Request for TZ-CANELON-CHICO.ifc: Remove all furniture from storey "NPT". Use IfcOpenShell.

First a look at what the model holds.

```python
import ifcopenshell
import ifcopenshell.util.element

model = ifcopenshell.open("TZ-CANELON-CHICO.ifc")
print(model.schema)
storey = next(s for s in model.by_type("IfcBuildingStorey") if s.Name == "NPT")
furniture = [e for e in ifcopenshell.util.element.get_decomposition(storey) if e.is_a("IfcFurnishingElement")]
seen = {}
for e in furniture:
    element_type = ifcopenshell.util.element.get_type(e)
    name = element_type.Name if element_type not in (None, e) else None
    seen[name] = seen.get(name, 0) + 1
for name, count in sorted(seen.items(), key=str):
    print(count, "x", name)
```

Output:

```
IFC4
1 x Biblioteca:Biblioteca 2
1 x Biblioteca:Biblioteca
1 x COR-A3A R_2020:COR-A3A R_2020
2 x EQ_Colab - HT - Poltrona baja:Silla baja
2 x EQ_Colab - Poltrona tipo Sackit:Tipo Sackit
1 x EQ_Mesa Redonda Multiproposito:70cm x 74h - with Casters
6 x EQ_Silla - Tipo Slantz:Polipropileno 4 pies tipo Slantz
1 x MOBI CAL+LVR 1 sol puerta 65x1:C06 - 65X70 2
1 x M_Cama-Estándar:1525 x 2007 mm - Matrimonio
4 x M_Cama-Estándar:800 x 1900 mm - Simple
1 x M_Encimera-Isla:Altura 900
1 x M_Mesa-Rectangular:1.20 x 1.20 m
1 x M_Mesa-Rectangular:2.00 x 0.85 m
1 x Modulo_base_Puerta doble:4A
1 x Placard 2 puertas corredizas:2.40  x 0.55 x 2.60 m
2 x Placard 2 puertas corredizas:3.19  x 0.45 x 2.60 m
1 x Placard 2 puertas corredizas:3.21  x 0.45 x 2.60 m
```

```python
import ifcopenshell
import ifcopenshell.api.root
import ifcopenshell.util.element

model = ifcopenshell.open("TZ-CANELON-CHICO.ifc")

storey = next(s for s in model.by_type("IfcBuildingStorey") if s.Name == "NPT")
furniture = [e for e in ifcopenshell.util.element.get_decomposition(storey) if e.is_a("IfcFurnishingElement")]

for e in furniture:
    ifcopenshell.api.root.remove_product(model, product=e)
print(len(furniture), "removed")

model.write("TZ-CANELON-CHICO-out.ifc")
```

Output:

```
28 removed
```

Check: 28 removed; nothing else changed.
